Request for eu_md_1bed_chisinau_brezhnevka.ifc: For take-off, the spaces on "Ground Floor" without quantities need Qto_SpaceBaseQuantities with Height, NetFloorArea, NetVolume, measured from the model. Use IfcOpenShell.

First a look at what the model holds.

```python
import ifcopenshell
import ifcopenshell.util.element
import ifcopenshell.util.unit

model = ifcopenshell.open("eu_md_1bed_chisinau_brezhnevka.ifc")
print(model.schema)
for unit_type in ("LENGTHUNIT", "AREAUNIT", "VOLUMEUNIT"):
    print(unit_type, ifcopenshell.util.unit.calculate_unit_scale(model, unit_type))
storey = next(s for s in model.by_type("IfcBuildingStorey") if s.Name == "Ground Floor")
spaces = [e for e in ifcopenshell.util.element.get_decomposition(storey) if e.is_a("IfcSpace")]
for e in sorted(spaces, key=lambda e: e.id()):
    print(e.id(), e.is_a(), e.Name, list(ifcopenshell.util.element.get_psets(e, qtos_only=True)), sep=" | ")
```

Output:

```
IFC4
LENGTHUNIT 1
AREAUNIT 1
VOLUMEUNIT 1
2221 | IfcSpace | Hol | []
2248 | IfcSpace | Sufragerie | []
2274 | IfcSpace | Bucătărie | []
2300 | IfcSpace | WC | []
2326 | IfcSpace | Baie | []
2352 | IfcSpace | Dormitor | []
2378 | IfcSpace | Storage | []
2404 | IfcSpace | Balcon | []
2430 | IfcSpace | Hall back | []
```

```python
import ifcopenshell
import ifcopenshell.api.pset
import ifcopenshell.geom
import ifcopenshell.util.element
import ifcopenshell.util.shape
import ifcopenshell.util.unit

model = ifcopenshell.open("eu_md_1bed_chisinau_brezhnevka.ifc")
unit_scale = ifcopenshell.util.unit.calculate_unit_scale(model)
area_scale = ifcopenshell.util.unit.calculate_unit_scale(model, "AREAUNIT")
volume_scale = ifcopenshell.util.unit.calculate_unit_scale(model, "VOLUMEUNIT")
settings = ifcopenshell.geom.settings()

storey = next(s for s in model.by_type("IfcBuildingStorey") if s.Name == "Ground Floor")
spaces = [e for e in ifcopenshell.util.element.get_decomposition(storey) if e.is_a("IfcSpace")]

for e in sorted(spaces, key=lambda e: e.id()):
    if ifcopenshell.util.element.get_psets(e, qtos_only=True, should_inherit=False):
        continue
    # Geometry comes back in metres, in the element's own axes.
    shape = ifcopenshell.geom.create_shape(settings, e)
    values = {
        "Height": ifcopenshell.util.shape.get_z(shape.geometry) / unit_scale,
        "NetFloorArea": ifcopenshell.util.shape.get_footprint_area(shape.geometry) / area_scale,
        "NetVolume": ifcopenshell.util.shape.get_volume(shape.geometry) / volume_scale,
    }
    qto = ifcopenshell.api.pset.add_qto(model, product=e, name="Qto_SpaceBaseQuantities")
    ifcopenshell.api.pset.edit_qto(model, qto=qto, properties=values)
    print(e.id(), {k: round(v, 3) for k, v in values.items()})

model.write("eu_md_1bed_chisinau_brezhnevka_edited.ifc")
```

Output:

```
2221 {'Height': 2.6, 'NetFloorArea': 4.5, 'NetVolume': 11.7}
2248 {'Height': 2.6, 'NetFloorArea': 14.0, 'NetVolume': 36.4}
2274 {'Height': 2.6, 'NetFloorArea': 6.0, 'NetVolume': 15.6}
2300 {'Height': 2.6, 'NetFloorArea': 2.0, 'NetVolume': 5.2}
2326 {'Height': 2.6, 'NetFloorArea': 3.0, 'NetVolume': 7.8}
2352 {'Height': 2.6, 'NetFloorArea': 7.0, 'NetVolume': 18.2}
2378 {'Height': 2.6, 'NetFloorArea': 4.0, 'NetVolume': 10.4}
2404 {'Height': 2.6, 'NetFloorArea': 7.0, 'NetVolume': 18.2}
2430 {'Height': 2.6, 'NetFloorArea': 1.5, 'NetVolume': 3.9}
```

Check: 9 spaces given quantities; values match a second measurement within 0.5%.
